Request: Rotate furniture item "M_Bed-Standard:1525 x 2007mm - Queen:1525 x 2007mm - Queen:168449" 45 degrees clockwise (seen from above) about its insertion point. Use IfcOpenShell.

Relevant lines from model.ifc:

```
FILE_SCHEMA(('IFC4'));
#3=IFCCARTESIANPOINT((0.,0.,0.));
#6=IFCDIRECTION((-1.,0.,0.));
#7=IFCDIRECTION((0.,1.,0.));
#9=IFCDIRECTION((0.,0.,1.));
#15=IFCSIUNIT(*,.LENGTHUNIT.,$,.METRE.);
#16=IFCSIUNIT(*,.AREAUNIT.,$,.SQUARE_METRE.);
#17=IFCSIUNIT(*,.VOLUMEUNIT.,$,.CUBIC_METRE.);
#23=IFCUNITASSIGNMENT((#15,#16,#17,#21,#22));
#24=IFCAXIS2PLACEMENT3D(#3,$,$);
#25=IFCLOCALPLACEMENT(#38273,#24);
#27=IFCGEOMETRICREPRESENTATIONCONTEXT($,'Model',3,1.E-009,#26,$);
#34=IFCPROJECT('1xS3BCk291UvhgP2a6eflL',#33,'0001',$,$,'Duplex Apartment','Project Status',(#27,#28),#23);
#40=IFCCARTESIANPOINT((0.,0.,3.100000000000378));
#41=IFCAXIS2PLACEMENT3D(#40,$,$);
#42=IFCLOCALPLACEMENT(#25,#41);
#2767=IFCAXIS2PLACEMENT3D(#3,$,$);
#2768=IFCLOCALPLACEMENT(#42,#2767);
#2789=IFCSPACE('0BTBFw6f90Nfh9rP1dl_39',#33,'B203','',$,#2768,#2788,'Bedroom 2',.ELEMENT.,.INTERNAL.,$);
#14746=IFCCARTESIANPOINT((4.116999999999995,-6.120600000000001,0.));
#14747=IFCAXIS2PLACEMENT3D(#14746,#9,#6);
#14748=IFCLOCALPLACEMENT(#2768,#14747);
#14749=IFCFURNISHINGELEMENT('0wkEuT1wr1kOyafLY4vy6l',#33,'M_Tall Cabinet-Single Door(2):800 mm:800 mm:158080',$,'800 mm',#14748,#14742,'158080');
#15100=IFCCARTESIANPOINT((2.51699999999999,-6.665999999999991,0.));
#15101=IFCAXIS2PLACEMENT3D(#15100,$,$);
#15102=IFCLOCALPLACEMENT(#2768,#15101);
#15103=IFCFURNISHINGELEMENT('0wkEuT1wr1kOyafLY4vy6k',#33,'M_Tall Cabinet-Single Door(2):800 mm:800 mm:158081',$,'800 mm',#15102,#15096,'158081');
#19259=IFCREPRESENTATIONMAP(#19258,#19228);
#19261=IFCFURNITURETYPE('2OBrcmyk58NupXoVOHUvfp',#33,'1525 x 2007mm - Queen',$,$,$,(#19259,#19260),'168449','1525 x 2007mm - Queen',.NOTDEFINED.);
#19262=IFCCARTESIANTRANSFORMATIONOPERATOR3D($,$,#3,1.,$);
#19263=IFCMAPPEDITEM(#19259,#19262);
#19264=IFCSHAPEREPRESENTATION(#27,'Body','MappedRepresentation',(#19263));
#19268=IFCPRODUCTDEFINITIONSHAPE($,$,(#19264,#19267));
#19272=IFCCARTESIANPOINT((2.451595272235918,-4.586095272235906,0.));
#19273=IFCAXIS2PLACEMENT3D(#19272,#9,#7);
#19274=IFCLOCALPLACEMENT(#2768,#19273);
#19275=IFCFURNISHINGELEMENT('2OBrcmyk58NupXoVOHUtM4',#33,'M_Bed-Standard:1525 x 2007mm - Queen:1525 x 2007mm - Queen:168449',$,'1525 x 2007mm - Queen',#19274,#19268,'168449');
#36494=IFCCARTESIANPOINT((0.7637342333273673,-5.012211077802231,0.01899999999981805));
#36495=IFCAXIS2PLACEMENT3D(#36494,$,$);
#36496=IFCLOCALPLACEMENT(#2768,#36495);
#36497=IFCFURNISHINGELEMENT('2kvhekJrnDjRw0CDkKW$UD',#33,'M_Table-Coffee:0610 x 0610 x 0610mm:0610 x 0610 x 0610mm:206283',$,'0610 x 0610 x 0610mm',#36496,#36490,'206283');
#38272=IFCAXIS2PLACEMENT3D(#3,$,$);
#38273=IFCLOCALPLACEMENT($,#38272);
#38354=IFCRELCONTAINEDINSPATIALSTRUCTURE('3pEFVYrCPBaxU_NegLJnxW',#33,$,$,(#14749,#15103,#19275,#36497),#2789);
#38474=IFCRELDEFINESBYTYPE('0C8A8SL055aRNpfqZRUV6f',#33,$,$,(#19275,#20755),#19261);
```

```python
import ifcopenshell
import ifcopenshell.api.geometry
import ifcopenshell.util.placement

model = ifcopenshell.open("model.ifc")

item = model.by_id(19275)
matrix = ifcopenshell.util.placement.get_local_placement(item.ObjectPlacement)
matrix = matrix @ ifcopenshell.util.placement.rotation(-45, "Z")
ifcopenshell.api.geometry.edit_object_placement(model, product=item, matrix=matrix, is_si=False)

print(ifcopenshell.util.placement.get_local_placement(item.ObjectPlacement).round(3) + 0.0)

model.write("model-out.ifc")
```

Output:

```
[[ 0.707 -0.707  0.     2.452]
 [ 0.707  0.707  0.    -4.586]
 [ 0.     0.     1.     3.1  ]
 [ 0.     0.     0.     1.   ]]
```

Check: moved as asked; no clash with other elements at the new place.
